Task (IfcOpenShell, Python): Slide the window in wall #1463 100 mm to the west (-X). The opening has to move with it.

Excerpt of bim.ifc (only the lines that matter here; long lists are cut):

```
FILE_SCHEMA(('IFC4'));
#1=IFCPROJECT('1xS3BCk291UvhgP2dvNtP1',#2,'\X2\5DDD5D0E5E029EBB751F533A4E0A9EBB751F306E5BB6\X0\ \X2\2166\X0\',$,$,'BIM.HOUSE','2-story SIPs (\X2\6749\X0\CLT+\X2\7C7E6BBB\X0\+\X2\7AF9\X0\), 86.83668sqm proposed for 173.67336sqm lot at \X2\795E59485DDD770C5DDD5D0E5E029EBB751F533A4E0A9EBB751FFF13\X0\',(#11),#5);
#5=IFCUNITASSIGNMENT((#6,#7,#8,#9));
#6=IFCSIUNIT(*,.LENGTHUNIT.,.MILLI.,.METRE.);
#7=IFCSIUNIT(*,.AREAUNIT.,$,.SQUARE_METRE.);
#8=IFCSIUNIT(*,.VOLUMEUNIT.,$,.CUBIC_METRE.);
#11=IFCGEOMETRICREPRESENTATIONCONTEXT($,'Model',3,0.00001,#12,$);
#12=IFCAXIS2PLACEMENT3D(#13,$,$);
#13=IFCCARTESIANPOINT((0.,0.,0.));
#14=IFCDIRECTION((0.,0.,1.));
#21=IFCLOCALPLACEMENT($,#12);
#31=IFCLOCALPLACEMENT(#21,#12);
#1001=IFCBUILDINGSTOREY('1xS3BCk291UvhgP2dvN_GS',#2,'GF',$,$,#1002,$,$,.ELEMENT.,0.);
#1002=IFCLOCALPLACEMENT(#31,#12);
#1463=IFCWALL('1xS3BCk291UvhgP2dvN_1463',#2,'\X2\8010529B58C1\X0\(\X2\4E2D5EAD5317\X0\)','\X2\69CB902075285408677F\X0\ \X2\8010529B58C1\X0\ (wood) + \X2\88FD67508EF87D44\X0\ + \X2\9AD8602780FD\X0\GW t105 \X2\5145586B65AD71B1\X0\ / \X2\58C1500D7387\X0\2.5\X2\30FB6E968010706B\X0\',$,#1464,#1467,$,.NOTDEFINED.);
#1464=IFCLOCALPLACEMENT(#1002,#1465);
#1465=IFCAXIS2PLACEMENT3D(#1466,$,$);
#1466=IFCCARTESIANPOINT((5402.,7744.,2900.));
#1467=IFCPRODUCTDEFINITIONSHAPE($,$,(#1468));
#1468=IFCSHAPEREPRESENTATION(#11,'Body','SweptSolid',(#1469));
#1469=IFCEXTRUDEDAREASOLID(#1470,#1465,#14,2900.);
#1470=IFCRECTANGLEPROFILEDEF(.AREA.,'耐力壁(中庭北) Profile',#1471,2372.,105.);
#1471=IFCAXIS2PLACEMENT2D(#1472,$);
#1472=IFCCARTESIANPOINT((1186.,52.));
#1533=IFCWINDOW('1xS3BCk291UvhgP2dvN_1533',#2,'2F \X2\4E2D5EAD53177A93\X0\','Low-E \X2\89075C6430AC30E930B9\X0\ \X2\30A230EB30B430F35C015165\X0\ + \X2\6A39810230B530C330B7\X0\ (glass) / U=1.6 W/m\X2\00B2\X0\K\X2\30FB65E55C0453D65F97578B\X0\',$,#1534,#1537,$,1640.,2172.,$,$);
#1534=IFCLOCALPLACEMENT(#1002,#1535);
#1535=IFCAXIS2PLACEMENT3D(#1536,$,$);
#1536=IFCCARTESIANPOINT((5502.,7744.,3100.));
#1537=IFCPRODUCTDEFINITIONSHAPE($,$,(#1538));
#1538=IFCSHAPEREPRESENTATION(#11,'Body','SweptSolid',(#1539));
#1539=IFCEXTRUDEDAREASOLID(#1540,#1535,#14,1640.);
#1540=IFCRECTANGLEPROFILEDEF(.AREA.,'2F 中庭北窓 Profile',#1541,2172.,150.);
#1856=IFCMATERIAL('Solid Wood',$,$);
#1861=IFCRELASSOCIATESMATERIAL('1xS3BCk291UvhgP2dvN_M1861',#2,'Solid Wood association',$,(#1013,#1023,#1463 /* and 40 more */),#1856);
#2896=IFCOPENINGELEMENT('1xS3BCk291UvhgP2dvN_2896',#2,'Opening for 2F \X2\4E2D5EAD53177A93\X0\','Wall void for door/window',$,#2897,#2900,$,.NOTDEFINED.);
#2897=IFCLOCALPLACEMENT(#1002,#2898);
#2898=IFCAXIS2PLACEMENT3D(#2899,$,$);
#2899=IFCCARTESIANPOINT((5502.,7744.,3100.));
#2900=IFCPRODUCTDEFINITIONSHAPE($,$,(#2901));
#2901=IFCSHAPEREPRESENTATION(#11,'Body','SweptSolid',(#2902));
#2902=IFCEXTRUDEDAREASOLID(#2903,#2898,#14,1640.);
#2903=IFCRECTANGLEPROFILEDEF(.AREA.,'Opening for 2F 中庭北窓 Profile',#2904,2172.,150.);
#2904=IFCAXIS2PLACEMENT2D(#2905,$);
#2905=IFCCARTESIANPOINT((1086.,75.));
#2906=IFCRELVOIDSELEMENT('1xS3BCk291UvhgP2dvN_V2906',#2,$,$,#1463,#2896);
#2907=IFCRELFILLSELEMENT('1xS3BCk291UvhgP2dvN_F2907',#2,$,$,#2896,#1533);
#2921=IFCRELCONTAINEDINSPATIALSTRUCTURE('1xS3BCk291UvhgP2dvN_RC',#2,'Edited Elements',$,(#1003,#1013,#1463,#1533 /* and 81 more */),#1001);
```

```python
import ifcopenshell
import ifcopenshell.api.geometry
import ifcopenshell.util.placement

model = ifcopenshell.open("bim.ifc")

window = model.by_id(1533)
opening = window.FillsVoids[0].RelatingOpeningElement
wall = opening.VoidsElements[0].RelatingBuildingElement

wall_matrix = ifcopenshell.util.placement.get_local_placement(wall.ObjectPlacement)
shift = wall_matrix[:3, 0] * -100.0
before = ifcopenshell.util.placement.get_local_placement(window.ObjectPlacement)[:3, 3].copy()

# The window is not placed relative to its opening, so move both.
for product in (opening, window):
    matrix = ifcopenshell.util.placement.get_local_placement(product.ObjectPlacement)
    matrix[:3, 3] += shift
    ifcopenshell.api.geometry.edit_object_placement(model, product=product, matrix=matrix, is_si=False)

after = ifcopenshell.util.placement.get_local_placement(window.ObjectPlacement)[:3, 3]
print("window moved by", (after - before).round(3) + 0.0)

model.write("bim_edited.ifc")
```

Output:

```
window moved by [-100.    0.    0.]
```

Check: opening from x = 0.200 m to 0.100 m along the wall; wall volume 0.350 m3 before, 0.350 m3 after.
